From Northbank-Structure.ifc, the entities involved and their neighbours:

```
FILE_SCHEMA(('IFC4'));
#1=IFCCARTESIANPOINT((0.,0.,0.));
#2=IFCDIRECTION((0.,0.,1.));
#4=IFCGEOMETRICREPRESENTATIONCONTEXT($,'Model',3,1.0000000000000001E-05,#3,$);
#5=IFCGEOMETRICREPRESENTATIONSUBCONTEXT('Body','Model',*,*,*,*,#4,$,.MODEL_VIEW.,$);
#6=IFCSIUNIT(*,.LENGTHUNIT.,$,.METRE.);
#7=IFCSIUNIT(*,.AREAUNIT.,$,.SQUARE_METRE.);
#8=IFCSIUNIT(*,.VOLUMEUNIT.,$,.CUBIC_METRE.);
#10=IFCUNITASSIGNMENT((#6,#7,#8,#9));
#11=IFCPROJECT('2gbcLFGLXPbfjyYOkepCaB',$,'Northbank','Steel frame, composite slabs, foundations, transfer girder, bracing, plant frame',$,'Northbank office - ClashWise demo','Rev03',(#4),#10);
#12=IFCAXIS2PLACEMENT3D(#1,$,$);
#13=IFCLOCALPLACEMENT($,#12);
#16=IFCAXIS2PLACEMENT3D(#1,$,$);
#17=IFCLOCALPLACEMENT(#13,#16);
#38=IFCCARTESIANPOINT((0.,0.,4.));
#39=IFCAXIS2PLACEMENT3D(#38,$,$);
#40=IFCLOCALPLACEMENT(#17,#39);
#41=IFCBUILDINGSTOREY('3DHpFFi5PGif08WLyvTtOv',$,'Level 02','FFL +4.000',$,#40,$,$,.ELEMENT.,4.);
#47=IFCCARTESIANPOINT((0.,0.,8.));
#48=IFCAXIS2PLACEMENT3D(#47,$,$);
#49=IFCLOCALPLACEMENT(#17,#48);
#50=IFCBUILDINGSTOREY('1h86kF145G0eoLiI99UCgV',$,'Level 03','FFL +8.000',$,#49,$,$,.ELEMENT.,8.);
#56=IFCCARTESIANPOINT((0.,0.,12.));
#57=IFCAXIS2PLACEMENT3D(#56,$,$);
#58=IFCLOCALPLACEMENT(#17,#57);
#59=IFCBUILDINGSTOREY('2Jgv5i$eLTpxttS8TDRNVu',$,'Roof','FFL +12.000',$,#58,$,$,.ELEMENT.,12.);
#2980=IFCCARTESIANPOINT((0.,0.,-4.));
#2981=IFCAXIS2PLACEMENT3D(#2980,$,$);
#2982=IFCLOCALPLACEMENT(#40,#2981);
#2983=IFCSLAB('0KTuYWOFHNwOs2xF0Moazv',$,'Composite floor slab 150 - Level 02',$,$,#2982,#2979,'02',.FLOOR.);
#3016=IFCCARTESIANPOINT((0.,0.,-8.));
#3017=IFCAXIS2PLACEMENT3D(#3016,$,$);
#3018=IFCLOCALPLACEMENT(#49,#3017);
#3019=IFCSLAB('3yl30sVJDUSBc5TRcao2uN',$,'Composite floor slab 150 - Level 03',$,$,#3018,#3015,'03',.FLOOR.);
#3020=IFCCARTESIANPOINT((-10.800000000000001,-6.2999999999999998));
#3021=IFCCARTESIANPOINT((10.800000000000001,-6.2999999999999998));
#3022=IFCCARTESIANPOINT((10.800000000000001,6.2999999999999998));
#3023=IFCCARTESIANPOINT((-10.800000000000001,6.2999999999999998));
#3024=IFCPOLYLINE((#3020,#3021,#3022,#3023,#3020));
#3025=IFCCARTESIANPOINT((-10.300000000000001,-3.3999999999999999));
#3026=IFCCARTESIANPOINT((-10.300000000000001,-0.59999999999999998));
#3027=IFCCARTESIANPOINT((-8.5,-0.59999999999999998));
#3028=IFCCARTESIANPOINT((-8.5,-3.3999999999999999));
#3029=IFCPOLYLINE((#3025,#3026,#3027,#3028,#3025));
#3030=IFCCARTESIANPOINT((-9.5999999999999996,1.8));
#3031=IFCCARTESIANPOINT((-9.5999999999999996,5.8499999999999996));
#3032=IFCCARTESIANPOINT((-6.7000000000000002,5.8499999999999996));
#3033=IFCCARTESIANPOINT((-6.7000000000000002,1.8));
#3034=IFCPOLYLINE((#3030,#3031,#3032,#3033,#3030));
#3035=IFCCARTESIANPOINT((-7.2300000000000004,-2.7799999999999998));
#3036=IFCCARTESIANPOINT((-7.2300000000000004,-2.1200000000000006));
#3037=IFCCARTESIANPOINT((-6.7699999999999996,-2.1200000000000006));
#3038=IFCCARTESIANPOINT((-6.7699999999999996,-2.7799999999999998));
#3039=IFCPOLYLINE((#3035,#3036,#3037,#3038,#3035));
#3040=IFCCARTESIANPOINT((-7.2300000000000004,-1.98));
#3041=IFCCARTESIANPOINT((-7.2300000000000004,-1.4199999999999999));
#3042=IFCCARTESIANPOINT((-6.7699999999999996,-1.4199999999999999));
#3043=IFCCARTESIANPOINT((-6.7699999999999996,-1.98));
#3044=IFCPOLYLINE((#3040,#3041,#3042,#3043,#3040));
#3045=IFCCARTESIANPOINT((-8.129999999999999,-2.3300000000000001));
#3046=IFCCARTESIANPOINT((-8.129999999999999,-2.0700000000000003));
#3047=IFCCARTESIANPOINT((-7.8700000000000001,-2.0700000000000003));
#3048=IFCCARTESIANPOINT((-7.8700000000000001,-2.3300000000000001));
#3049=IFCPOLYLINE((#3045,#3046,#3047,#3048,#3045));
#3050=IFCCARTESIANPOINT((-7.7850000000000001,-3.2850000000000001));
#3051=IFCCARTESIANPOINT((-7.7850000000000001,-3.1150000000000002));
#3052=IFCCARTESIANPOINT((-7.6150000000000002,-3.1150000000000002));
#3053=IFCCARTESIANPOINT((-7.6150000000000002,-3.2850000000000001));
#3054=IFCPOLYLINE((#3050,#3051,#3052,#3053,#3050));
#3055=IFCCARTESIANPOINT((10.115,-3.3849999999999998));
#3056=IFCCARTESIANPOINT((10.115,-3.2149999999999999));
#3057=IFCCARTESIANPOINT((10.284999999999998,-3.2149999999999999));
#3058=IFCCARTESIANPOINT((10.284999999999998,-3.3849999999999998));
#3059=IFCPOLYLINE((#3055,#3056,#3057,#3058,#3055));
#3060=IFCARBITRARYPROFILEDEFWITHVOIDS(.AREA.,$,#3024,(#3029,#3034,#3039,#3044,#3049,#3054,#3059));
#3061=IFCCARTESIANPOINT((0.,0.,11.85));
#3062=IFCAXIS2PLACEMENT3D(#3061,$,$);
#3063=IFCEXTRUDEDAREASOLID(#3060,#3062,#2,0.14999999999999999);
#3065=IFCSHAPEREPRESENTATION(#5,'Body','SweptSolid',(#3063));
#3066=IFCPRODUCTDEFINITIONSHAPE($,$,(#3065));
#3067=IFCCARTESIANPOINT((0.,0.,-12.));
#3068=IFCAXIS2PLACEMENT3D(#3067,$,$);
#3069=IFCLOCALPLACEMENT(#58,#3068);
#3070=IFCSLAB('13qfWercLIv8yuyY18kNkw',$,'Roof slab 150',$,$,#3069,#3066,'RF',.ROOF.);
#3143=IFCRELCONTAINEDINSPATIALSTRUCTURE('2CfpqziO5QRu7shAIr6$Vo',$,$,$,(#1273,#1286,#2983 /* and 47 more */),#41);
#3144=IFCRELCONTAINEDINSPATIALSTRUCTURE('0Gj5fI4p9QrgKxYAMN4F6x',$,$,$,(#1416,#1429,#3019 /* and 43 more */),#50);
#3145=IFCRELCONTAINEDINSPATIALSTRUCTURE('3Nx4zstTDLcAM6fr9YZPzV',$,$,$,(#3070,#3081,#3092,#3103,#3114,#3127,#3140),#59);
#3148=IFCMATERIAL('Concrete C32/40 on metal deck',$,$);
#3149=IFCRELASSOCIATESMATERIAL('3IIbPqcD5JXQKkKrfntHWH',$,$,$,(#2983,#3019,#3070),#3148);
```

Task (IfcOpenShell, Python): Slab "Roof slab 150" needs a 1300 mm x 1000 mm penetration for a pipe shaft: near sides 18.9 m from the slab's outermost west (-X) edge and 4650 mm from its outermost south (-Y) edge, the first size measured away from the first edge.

```python
import numpy as np
import ifcopenshell
import ifcopenshell.api.feature
import ifcopenshell.api.geometry
import ifcopenshell.api.root
import ifcopenshell.geom
import ifcopenshell.util.placement
import ifcopenshell.util.representation
import ifcopenshell.util.shape
import ifcopenshell.util.unit

model = ifcopenshell.open("Northbank-Structure.ifc")
unit_scale = ifcopenshell.util.unit.calculate_unit_scale(model)
settings = ifcopenshell.geom.settings()


def volume(element):
    """Net volume in cubic metres, openings subtracted."""
    shape = ifcopenshell.geom.create_shape(settings, element)
    return ifcopenshell.util.shape.get_volume(shape.geometry)


slab = model.by_id(3070)
before = volume(slab)

# Extent in the slab's own axes, in metres. The edges named are its -X and -Y sides.
slab_shape = ifcopenshell.geom.create_shape(settings, slab)
vertices = ifcopenshell.util.shape.get_vertices(slab_shape.geometry)
x_min, y_min, bottom = vertices.min(axis=0)
top = vertices[:, 2].max()

opening = ifcopenshell.api.root.create_entity(model, ifc_class="IfcOpeningElement", name="Pipe shaft opening", predefined_type="OPENING")
context = ifcopenshell.util.representation.get_context(model, "Model", "Body", "MODEL_VIEW")
width, depth = 1.3, 1
outline = [(0.0, 0.0), (width, 0.0), (width, depth), (0.0, depth), (0.0, 0.0)]
# Overshoot both faces by 50 mm so the cut is clean.
shape = ifcopenshell.api.geometry.add_slab_representation(
    model, context=context, depth=top - bottom + 0.1, polyline=outline
)
ifcopenshell.api.geometry.assign_representation(model, product=opening, representation=shape)

matrix = ifcopenshell.util.placement.get_local_placement(slab.ObjectPlacement)
matrix[:, 3] = matrix @ np.append(np.array([x_min + 18.9, y_min + 4.65, bottom - 0.05]) / unit_scale, 1.0)
ifcopenshell.api.geometry.edit_object_placement(model, product=opening, matrix=matrix, is_si=False)
ifcopenshell.api.feature.add_feature(model, feature=opening, element=slab)

after = volume(slab)

print(f"slab volume {before:.3f} -> {after:.3f} m3")

model.write("Northbank-Structure_edited.ifc")
```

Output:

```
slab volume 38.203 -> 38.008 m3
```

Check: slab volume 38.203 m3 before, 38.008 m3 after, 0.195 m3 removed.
